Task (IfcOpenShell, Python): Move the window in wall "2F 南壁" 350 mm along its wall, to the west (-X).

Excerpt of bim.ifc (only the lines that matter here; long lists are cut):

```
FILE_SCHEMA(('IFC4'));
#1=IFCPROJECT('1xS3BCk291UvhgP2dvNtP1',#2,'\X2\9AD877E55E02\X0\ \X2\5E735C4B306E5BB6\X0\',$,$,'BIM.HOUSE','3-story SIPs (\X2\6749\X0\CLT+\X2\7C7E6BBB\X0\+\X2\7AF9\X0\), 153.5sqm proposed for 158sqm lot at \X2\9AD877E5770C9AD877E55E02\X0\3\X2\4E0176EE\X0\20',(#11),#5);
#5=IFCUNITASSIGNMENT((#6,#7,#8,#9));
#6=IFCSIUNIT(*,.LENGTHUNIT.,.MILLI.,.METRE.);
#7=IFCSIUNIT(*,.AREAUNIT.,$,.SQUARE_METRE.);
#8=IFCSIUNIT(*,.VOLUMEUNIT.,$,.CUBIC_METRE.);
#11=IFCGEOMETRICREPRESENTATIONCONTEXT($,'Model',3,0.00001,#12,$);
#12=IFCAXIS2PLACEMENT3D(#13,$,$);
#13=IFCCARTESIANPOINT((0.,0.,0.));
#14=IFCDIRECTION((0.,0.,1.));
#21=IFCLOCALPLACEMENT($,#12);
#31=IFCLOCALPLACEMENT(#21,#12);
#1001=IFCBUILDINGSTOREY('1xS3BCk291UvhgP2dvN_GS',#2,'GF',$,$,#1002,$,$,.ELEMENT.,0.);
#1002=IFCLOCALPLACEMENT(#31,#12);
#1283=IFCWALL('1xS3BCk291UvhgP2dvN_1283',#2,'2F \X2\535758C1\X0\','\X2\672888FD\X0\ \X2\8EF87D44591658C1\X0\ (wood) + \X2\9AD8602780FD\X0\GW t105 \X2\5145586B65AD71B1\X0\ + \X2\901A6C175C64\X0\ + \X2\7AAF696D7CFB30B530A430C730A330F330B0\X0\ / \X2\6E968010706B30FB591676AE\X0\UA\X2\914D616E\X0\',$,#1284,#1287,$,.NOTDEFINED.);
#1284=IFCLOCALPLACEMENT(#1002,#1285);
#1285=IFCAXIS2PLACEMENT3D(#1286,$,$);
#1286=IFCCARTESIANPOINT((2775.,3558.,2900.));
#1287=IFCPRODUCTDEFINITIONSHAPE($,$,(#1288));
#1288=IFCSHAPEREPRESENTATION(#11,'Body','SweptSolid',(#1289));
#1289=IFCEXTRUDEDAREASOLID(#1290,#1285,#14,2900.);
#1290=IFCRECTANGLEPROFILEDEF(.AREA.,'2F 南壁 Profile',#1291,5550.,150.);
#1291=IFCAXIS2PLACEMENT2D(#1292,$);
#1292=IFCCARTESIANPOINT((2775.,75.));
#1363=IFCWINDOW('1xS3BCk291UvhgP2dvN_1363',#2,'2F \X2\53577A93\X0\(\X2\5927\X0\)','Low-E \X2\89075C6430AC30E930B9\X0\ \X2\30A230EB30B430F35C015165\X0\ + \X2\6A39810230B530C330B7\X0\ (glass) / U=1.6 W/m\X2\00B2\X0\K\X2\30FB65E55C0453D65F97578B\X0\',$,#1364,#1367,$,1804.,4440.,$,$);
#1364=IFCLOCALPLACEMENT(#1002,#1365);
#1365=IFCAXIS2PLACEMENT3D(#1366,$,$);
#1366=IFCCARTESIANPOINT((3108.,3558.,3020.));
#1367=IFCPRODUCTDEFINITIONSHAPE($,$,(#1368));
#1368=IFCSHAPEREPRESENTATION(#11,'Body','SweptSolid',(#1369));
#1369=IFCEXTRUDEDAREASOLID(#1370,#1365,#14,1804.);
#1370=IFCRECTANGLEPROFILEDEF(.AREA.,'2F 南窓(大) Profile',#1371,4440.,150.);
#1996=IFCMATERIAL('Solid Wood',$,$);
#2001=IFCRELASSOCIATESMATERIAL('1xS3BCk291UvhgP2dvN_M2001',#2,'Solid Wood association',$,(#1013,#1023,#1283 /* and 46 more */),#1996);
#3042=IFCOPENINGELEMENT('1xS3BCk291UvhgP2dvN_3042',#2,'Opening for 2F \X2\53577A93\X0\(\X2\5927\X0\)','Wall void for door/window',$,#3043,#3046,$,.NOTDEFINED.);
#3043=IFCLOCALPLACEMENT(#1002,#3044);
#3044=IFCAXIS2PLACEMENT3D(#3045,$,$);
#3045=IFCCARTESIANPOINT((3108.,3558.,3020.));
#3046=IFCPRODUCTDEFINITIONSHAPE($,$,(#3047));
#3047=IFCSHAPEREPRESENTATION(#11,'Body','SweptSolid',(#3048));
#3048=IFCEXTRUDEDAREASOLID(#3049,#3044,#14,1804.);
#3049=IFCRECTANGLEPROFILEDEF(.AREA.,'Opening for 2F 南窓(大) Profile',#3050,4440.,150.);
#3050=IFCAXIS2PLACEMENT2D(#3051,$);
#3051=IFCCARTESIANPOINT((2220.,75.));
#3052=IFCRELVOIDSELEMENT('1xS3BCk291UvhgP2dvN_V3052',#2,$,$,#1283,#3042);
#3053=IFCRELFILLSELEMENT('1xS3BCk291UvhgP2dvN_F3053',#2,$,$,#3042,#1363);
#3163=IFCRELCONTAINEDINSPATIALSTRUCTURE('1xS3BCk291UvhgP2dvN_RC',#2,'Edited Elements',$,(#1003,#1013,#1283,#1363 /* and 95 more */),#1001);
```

```python
import ifcopenshell
import ifcopenshell.api.geometry
import ifcopenshell.util.placement
import ifcopenshell.util.unit

model = ifcopenshell.open("bim.ifc")
unit_scale = ifcopenshell.util.unit.calculate_unit_scale(model)

window = model.by_id(1363)
opening = window.FillsVoids[0].RelatingOpeningElement
wall = opening.VoidsElements[0].RelatingBuildingElement

wall_matrix = ifcopenshell.util.placement.get_local_placement(wall.ObjectPlacement)
shift = wall_matrix[:3, 0] * -0.35 / unit_scale
before = ifcopenshell.util.placement.get_local_placement(window.ObjectPlacement)[:3, 3].copy()

# The window is not placed relative to its opening, so move both.
for product in (opening, window):
    matrix = ifcopenshell.util.placement.get_local_placement(product.ObjectPlacement)
    matrix[:3, 3] += shift
    ifcopenshell.api.geometry.edit_object_placement(model, product=product, matrix=matrix, is_si=False)

after = ifcopenshell.util.placement.get_local_placement(window.ObjectPlacement)[:3, 3]
print("window moved by", (after - before).round(3) + 0.0)

model.write("bim_rev.ifc")
```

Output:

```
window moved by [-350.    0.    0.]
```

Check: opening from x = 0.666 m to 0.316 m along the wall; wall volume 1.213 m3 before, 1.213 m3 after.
